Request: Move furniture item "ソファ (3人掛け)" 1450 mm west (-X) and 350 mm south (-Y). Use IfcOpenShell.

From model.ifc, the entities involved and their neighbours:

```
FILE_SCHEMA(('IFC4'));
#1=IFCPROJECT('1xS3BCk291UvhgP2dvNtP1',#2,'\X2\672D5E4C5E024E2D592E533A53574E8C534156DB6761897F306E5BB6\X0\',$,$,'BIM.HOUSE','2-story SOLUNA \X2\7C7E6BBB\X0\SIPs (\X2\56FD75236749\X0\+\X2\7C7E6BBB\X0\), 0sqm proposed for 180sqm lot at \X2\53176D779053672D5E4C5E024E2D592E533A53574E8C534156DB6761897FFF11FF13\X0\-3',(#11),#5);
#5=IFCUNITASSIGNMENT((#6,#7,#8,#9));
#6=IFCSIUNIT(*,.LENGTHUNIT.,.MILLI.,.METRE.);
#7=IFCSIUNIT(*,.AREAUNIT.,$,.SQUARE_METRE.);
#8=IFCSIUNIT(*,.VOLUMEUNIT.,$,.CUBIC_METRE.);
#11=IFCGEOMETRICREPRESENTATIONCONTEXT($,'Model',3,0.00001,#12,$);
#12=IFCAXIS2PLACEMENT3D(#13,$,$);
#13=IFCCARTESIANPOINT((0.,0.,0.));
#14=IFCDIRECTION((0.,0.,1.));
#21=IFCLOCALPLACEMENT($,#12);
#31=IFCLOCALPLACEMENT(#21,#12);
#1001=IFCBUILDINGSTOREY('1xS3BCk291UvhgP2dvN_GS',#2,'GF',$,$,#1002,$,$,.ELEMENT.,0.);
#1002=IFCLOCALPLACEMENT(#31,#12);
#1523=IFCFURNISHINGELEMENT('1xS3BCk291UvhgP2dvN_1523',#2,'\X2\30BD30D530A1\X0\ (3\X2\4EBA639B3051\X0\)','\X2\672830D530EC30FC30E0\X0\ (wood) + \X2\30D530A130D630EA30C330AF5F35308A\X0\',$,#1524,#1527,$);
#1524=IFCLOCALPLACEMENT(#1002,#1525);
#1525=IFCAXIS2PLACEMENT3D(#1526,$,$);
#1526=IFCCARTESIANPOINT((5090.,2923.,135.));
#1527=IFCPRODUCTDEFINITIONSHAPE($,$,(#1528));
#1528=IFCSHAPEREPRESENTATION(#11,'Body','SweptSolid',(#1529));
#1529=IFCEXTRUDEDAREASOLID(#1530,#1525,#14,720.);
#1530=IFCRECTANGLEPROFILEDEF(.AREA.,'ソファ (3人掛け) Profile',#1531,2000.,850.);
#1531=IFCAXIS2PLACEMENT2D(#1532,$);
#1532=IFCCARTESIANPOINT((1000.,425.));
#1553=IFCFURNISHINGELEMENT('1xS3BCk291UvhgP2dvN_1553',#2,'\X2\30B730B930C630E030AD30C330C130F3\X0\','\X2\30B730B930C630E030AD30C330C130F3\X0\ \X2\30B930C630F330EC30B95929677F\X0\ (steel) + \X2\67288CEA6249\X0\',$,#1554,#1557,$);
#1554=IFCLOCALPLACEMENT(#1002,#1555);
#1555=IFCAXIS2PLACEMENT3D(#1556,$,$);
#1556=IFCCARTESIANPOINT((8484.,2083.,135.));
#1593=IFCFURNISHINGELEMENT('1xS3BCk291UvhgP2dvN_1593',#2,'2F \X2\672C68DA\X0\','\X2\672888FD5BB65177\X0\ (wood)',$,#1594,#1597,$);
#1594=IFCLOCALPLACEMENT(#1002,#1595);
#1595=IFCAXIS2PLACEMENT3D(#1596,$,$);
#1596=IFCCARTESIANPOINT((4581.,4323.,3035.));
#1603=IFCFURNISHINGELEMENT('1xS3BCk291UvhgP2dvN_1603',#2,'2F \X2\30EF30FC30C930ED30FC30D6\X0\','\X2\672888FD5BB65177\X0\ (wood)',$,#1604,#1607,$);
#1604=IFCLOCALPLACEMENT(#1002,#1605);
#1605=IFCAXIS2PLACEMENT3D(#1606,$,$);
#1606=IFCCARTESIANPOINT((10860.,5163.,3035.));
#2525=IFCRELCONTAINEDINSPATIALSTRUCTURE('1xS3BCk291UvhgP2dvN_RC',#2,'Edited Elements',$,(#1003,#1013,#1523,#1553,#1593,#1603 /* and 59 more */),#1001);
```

```python
import ifcopenshell
import ifcopenshell.api.geometry
import ifcopenshell.util.placement
import ifcopenshell.util.unit

model = ifcopenshell.open("model.ifc")
unit_scale = ifcopenshell.util.unit.calculate_unit_scale(model)

item = model.by_id(1523)
matrix = ifcopenshell.util.placement.get_local_placement(item.ObjectPlacement)
matrix[0, 3] -= 1.45 / unit_scale
matrix[1, 3] -= 0.35 / unit_scale
ifcopenshell.api.geometry.edit_object_placement(model, product=item, matrix=matrix, is_si=False)

print(ifcopenshell.util.placement.get_local_placement(item.ObjectPlacement).round(3) + 0.0)

model.write("model_rev.ifc")
```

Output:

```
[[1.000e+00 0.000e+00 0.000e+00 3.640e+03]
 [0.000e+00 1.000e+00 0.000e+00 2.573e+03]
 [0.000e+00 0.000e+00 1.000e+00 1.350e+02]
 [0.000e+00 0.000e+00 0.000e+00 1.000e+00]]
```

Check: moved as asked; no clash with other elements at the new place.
